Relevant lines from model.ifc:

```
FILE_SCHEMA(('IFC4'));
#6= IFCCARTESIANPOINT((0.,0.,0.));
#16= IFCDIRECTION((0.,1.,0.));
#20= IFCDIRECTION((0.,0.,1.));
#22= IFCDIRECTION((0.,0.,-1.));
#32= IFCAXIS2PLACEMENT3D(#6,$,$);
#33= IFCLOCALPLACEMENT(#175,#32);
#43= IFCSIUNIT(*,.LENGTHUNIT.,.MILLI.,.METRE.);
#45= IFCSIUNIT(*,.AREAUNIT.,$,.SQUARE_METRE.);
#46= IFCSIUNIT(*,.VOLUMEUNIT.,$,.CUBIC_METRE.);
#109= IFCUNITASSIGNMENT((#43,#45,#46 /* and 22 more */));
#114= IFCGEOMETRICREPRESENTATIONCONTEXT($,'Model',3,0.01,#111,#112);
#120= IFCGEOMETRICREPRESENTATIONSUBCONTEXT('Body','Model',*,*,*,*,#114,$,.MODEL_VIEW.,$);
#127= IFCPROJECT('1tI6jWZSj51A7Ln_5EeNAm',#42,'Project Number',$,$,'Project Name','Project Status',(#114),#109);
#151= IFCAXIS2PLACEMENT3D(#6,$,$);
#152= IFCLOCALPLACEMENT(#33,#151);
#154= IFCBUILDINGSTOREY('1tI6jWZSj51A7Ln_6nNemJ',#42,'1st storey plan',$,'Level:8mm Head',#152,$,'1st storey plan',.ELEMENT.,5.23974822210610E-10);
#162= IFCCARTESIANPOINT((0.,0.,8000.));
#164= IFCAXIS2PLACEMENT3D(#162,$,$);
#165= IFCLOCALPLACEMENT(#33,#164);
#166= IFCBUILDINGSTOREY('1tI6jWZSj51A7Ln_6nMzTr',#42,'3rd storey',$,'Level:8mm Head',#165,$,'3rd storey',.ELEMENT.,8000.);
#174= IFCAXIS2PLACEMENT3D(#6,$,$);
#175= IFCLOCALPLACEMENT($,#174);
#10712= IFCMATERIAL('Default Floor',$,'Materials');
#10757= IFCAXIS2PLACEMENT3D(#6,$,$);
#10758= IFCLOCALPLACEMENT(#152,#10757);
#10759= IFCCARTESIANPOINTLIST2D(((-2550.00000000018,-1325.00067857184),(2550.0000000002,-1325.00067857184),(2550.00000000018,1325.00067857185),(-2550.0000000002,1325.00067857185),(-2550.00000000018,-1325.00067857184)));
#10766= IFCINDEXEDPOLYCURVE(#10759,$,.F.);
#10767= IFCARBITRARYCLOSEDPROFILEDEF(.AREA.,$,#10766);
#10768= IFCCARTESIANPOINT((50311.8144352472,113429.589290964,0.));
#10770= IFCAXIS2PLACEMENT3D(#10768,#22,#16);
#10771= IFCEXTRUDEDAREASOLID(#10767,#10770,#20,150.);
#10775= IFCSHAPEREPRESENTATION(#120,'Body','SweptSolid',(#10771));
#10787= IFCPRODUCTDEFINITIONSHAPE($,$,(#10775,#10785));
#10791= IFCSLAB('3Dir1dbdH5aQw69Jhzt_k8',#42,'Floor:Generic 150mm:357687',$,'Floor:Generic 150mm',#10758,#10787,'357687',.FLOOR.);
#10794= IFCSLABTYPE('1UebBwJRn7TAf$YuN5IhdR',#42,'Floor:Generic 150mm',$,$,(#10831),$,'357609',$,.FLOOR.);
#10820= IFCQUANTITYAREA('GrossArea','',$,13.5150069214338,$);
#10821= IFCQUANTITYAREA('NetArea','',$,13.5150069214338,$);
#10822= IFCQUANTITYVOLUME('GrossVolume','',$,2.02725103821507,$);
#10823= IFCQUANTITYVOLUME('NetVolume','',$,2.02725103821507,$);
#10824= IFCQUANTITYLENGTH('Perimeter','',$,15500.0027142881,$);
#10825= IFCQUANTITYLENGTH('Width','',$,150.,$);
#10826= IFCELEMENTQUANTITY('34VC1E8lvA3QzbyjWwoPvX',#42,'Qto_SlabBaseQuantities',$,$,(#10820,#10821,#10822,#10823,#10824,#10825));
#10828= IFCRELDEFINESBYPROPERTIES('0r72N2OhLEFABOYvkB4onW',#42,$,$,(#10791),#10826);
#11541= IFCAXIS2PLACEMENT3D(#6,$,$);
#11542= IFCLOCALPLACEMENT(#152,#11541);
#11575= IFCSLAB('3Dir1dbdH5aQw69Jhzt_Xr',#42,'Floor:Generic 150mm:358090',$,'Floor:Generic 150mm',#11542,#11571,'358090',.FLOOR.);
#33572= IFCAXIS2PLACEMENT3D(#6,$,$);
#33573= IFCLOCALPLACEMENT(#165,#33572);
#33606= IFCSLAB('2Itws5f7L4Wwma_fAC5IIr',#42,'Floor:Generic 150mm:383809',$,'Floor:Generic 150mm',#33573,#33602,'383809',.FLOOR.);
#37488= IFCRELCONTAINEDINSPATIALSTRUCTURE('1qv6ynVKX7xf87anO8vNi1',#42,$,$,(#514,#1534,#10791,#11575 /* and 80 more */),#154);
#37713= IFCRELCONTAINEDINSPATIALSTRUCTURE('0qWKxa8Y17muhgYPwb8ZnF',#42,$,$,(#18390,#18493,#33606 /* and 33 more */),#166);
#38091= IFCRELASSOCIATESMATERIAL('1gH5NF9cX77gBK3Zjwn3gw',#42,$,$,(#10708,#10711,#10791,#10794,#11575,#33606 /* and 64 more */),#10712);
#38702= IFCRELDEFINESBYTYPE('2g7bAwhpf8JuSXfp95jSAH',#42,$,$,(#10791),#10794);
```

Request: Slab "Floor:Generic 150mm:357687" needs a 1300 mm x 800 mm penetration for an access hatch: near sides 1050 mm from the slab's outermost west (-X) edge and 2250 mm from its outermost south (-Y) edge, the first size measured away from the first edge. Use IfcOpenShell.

```python
import numpy as np
import ifcopenshell
import ifcopenshell.api.feature
import ifcopenshell.api.geometry
import ifcopenshell.api.pset
import ifcopenshell.api.root
import ifcopenshell.geom
import ifcopenshell.util.element
import ifcopenshell.util.placement
import ifcopenshell.util.representation
import ifcopenshell.util.shape
import ifcopenshell.util.unit

model = ifcopenshell.open("model.ifc")
unit_scale = ifcopenshell.util.unit.calculate_unit_scale(model)
area_scale = ifcopenshell.util.unit.calculate_unit_scale(model, "AREAUNIT")
volume_scale = ifcopenshell.util.unit.calculate_unit_scale(model, "VOLUMEUNIT")
settings = ifcopenshell.geom.settings()


def volume(element):
    """Net volume in cubic metres, openings subtracted."""
    shape = ifcopenshell.geom.create_shape(settings, element)
    return ifcopenshell.util.shape.get_volume(shape.geometry)


slab = model.by_guid("3Dir1dbdH5aQw69Jhzt_k8")
before = volume(slab)

# Extent in the slab's own axes, in metres. The edges named are its -X and -Y sides.
slab_shape = ifcopenshell.geom.create_shape(settings, slab)
vertices = ifcopenshell.util.shape.get_vertices(slab_shape.geometry)
x_min, y_min, bottom = vertices.min(axis=0)
top = vertices[:, 2].max()

opening = ifcopenshell.api.root.create_entity(model, ifc_class="IfcOpeningElement", name="Access hatch opening", predefined_type="OPENING")
context = ifcopenshell.util.representation.get_context(model, "Model", "Body", "MODEL_VIEW")
width, depth = 1.3, 0.8
outline = [(0.0, 0.0), (width, 0.0), (width, depth), (0.0, depth), (0.0, 0.0)]
# Overshoot both faces by 50 mm so the cut is clean.
shape = ifcopenshell.api.geometry.add_slab_representation(
    model, context=context, depth=top - bottom + 0.1, polyline=outline
)
ifcopenshell.api.geometry.assign_representation(model, product=opening, representation=shape)

matrix = ifcopenshell.util.placement.get_local_placement(slab.ObjectPlacement)
matrix[:, 3] = matrix @ np.append(np.array([x_min + 1.05, y_min + 2.25, bottom - 0.05]) / unit_scale, 1.0)
ifcopenshell.api.geometry.edit_object_placement(model, product=opening, matrix=matrix, is_si=False)
ifcopenshell.api.feature.add_feature(model, feature=opening, element=slab)

after = volume(slab)

# Update the slab's stored quantities.
qto = model.by_id(ifcopenshell.util.element.get_pset(slab, "Qto_SlabBaseQuantities", should_inherit=False)["id"])
ifcopenshell.api.pset.edit_qto(model, qto=qto, properties={
    "NetArea": after / (top - bottom) / area_scale,
    "NetVolume": after / volume_scale,
})

print(f"slab volume {before:.3f} -> {after:.3f} m3")

model.write("model-out.ifc")
```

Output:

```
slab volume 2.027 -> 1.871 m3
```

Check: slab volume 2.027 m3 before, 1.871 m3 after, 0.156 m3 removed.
